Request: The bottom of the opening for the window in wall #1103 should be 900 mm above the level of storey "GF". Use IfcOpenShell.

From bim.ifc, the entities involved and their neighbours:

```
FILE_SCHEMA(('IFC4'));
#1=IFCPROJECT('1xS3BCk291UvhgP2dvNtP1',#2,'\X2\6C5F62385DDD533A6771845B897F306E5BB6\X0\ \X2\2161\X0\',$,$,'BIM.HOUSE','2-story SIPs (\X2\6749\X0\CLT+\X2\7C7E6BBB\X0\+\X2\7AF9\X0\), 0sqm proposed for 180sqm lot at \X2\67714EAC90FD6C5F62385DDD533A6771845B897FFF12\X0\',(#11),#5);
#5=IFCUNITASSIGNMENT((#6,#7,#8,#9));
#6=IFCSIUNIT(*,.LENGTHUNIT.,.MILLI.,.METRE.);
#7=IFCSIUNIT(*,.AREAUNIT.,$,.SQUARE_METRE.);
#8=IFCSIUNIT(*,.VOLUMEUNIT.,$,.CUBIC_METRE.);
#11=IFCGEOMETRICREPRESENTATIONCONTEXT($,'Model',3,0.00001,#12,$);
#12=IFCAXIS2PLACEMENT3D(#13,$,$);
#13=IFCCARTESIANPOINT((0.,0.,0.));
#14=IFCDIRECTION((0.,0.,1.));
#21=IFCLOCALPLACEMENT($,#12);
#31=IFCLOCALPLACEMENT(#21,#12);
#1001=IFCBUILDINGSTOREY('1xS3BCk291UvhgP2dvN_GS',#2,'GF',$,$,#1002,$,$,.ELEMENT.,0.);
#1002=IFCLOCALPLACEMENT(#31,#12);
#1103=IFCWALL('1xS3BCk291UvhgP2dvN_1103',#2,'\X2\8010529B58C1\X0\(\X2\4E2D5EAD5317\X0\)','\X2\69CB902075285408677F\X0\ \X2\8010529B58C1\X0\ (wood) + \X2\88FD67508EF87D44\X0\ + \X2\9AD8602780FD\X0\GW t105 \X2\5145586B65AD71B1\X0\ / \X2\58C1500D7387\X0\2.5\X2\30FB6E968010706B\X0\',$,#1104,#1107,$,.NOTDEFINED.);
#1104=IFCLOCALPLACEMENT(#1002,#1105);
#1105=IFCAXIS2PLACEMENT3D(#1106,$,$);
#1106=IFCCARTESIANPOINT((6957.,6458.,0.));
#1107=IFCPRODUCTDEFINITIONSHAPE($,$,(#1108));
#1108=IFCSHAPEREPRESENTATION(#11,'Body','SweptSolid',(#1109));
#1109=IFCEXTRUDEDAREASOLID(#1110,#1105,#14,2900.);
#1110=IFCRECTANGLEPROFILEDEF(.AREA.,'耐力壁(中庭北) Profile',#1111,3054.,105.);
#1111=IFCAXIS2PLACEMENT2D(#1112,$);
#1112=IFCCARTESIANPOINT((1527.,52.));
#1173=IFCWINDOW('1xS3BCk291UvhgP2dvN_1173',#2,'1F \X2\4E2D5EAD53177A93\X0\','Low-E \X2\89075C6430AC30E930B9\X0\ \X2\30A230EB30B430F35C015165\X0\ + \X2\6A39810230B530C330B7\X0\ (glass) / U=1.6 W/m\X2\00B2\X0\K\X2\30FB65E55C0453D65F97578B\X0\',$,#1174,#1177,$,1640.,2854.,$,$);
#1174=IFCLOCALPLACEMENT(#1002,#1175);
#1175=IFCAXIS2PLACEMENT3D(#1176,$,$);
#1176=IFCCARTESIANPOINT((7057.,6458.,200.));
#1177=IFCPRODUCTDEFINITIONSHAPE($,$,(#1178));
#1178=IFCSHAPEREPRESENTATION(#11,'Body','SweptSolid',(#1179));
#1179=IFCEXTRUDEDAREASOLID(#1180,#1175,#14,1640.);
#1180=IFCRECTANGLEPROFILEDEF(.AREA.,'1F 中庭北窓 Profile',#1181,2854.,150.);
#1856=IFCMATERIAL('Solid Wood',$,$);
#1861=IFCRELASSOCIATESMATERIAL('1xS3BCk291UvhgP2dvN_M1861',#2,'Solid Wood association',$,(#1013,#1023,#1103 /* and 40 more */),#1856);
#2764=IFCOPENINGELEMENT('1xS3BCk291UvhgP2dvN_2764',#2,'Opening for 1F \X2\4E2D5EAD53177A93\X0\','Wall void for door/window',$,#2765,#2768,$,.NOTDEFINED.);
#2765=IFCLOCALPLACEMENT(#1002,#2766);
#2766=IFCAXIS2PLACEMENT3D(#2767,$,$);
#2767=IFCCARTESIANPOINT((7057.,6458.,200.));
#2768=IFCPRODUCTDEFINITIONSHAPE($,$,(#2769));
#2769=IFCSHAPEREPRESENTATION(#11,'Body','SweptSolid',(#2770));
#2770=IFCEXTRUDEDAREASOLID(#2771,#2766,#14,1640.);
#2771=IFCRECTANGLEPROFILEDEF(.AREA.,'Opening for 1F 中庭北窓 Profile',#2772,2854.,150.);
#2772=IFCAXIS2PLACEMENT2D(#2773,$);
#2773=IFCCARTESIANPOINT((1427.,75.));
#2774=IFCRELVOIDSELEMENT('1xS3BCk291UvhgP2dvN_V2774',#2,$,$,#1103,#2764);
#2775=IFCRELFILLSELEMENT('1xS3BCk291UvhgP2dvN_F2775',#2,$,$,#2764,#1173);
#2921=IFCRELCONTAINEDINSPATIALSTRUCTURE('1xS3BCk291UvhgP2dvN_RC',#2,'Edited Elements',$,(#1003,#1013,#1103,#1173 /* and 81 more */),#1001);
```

```python
import numpy as np
import ifcopenshell
import ifcopenshell.api.geometry
import ifcopenshell.geom
import ifcopenshell.util.element
import ifcopenshell.util.placement
import ifcopenshell.util.shape
import ifcopenshell.util.unit

model = ifcopenshell.open("bim.ifc")
unit_scale = ifcopenshell.util.unit.calculate_unit_scale(model)

window = model.by_guid("1xS3BCk291UvhgP2dvN_1173")
opening = window.FillsVoids[0].RelatingOpeningElement
storey = ifcopenshell.util.element.get_container(window, ifc_class="IfcBuildingStorey")
level = ifcopenshell.util.placement.get_local_placement(storey.ObjectPlacement)[2, 3]

# The opening's origin need not be at the sill, so measure its lowest point.
shape = ifcopenshell.geom.create_shape(ifcopenshell.geom.settings(), opening)
bottom = ifcopenshell.util.shape.get_shape_bottom_elevation(shape, shape.geometry) / unit_scale
dz = level + 0.9 / unit_scale - bottom

shift = np.array([0.0, 0.0, dz])
# The window is not placed relative to its opening, so move both.
for product in (opening, window):
    matrix = ifcopenshell.util.placement.get_local_placement(product.ObjectPlacement)
    matrix[:3, 3] += shift
    ifcopenshell.api.geometry.edit_object_placement(model, product=product, matrix=matrix, is_si=False)

print(f"moved by {dz * unit_scale:+.3f} m")

model.write("bim_updated.ifc")
```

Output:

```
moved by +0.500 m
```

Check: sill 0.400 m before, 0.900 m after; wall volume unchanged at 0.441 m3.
